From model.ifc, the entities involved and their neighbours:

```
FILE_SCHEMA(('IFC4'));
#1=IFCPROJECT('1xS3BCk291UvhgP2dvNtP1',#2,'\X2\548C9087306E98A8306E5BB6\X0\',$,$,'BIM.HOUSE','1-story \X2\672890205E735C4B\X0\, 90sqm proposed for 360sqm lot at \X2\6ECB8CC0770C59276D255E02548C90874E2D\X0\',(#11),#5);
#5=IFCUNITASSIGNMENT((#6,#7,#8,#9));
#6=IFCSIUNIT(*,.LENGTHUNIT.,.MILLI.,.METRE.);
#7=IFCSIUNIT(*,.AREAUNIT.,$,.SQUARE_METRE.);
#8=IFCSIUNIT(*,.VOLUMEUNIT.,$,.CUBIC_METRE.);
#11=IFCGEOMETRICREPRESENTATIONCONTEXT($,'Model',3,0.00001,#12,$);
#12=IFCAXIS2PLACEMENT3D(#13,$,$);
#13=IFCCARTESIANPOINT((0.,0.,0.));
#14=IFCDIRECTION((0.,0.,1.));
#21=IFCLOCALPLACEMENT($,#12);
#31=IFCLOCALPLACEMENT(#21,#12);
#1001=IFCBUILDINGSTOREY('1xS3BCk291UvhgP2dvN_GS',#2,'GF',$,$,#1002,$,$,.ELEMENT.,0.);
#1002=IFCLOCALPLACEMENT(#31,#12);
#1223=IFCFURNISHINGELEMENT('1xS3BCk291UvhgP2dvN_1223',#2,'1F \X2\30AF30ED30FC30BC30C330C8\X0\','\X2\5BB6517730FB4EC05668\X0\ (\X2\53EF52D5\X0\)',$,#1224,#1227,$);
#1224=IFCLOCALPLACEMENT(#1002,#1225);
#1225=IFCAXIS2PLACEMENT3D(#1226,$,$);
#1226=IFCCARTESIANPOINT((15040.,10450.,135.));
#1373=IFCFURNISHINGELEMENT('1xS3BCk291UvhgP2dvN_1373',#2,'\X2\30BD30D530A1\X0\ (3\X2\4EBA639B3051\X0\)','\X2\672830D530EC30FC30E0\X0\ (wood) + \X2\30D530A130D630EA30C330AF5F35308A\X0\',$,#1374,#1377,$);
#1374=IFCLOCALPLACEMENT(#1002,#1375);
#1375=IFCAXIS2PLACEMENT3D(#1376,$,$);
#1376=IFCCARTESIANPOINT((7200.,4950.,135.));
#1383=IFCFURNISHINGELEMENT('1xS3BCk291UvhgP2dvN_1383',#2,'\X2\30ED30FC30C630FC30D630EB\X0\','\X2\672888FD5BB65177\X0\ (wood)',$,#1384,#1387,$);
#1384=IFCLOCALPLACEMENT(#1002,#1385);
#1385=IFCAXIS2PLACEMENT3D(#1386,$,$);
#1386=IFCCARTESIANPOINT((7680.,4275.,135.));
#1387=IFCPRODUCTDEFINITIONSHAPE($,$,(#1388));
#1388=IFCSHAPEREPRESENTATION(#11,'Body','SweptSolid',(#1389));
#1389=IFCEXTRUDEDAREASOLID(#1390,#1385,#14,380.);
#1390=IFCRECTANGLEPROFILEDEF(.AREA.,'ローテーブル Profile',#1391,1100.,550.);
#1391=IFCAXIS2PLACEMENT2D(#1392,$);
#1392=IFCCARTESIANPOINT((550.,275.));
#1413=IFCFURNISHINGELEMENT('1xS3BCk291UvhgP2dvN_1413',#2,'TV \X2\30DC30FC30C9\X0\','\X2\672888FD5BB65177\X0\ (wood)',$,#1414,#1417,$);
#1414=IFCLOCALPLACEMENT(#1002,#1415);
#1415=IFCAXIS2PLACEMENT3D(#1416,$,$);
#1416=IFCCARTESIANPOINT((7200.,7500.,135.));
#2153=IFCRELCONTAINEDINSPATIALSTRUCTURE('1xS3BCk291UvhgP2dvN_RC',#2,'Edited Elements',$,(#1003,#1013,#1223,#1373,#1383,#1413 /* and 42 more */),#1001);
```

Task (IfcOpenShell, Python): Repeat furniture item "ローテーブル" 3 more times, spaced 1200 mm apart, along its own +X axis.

```python
import ifcopenshell
import ifcopenshell.api.geometry
import ifcopenshell.api.root
import ifcopenshell.util.element
import ifcopenshell.util.placement
import ifcopenshell.util.unit

model = ifcopenshell.open("model.ifc")
unit_scale = ifcopenshell.util.unit.calculate_unit_scale(model)


def reuse_history(source, copy):
    """copy_class also copies each property set's owner history, people and application; keep the originals."""
    for rel in copy.IsDefinedBy:
        if rel.is_a("IfcRelDefinesByProperties") and (history := rel.RelatingPropertyDefinition.OwnerHistory):
            rel.RelatingPropertyDefinition.OwnerHistory = source.OwnerHistory
            ifcopenshell.util.element.remove_deep2(model, history)


source = model.by_guid("1xS3BCk291UvhgP2dvN_1383")
base = ifcopenshell.util.placement.get_local_placement(source.ObjectPlacement)
step = base[:3, 0] * 1.2 / unit_scale

for i in range(1, 4):
    copy = ifcopenshell.api.root.copy_class(model, product=source)
    copy.Representation = ifcopenshell.util.element.copy_deep(
        model, source.Representation, exclude=["IfcGeometricRepresentationContext", "IfcRepresentationMap"]
    )
    reuse_history(source, copy)
    matrix = base.copy()
    matrix[:3, 3] += i * step
    print("added at", matrix[:3, 3].round(3) + 0.0)
    ifcopenshell.api.geometry.edit_object_placement(model, product=copy, matrix=matrix, is_si=False)

model.write("model_rev.ifc")
```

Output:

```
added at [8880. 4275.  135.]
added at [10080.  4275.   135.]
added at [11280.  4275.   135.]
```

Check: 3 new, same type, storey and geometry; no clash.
